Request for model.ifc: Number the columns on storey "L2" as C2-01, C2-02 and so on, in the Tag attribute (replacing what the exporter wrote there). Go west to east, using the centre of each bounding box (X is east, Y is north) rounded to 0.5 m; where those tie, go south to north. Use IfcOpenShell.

First a look at what the model holds.

```python
import ifcopenshell
import ifcopenshell.util.element
import ifcopenshell.util.placement

model = ifcopenshell.open("model.ifc")
print(model.schema)
storey = next(s for s in model.by_type("IfcBuildingStorey") if s.Name == "L2")
columns = [e for e in ifcopenshell.util.element.get_decomposition(storey) if e.is_a("IfcColumn")]
for e in sorted(columns, key=lambda e: e.id()):
    origin = ifcopenshell.util.placement.get_local_placement(e.ObjectPlacement)[:3, 3]
    print(e.id(), e.Tag, e.Name, origin.round(2) + 0.0, sep=" | ")
```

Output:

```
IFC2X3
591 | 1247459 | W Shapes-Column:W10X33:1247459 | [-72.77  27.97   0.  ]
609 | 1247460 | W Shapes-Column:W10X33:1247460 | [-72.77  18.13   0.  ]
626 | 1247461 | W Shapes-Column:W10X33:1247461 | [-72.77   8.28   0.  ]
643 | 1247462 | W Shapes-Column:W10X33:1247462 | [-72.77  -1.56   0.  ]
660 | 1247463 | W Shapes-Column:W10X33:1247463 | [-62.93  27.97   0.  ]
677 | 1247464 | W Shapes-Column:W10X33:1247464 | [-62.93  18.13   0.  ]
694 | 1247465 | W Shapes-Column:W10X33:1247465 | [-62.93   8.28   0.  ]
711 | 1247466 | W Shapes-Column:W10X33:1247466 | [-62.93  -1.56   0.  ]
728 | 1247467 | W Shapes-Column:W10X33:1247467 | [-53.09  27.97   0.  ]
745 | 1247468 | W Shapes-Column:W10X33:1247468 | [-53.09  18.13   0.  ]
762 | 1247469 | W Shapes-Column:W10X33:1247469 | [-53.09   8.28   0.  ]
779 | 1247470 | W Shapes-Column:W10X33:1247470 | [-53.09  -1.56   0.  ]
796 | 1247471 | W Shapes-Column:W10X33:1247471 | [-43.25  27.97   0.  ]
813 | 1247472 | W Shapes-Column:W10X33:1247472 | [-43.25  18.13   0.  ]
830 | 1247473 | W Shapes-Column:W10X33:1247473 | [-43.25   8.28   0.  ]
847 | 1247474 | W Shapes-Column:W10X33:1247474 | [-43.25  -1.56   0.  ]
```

```python
import ifcopenshell
import ifcopenshell.geom
import ifcopenshell.util.element
import ifcopenshell.util.shape

model = ifcopenshell.open("model.ifc")
settings = ifcopenshell.geom.settings()
settings.set("use-world-coords", True)


def centre(element):
    shape = ifcopenshell.geom.create_shape(settings, element)
    return ifcopenshell.util.shape.get_bbox_centroid(shape.geometry)


storey = next(s for s in model.by_type("IfcBuildingStorey") if s.Name == "L2")
columns = [e for e in ifcopenshell.util.element.get_decomposition(storey) if e.is_a("IfcColumn")]

# Insertion points can sit at a corner or the storey origin, so sort by the geometry (in metres).
centres = {e: centre(e) for e in columns}
columns.sort(key=lambda e: (round(centres[e][0] / 0.5), centres[e][1]))

for i, e in enumerate(columns, start=1):
    number = f"C2-{i:02d}"
    e.Tag = number
    print(e.id(), number)

model.write("model_edited.ifc")
```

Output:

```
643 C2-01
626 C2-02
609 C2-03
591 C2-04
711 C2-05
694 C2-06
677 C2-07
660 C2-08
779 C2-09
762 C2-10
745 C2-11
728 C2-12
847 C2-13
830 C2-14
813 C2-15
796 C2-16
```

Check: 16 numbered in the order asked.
